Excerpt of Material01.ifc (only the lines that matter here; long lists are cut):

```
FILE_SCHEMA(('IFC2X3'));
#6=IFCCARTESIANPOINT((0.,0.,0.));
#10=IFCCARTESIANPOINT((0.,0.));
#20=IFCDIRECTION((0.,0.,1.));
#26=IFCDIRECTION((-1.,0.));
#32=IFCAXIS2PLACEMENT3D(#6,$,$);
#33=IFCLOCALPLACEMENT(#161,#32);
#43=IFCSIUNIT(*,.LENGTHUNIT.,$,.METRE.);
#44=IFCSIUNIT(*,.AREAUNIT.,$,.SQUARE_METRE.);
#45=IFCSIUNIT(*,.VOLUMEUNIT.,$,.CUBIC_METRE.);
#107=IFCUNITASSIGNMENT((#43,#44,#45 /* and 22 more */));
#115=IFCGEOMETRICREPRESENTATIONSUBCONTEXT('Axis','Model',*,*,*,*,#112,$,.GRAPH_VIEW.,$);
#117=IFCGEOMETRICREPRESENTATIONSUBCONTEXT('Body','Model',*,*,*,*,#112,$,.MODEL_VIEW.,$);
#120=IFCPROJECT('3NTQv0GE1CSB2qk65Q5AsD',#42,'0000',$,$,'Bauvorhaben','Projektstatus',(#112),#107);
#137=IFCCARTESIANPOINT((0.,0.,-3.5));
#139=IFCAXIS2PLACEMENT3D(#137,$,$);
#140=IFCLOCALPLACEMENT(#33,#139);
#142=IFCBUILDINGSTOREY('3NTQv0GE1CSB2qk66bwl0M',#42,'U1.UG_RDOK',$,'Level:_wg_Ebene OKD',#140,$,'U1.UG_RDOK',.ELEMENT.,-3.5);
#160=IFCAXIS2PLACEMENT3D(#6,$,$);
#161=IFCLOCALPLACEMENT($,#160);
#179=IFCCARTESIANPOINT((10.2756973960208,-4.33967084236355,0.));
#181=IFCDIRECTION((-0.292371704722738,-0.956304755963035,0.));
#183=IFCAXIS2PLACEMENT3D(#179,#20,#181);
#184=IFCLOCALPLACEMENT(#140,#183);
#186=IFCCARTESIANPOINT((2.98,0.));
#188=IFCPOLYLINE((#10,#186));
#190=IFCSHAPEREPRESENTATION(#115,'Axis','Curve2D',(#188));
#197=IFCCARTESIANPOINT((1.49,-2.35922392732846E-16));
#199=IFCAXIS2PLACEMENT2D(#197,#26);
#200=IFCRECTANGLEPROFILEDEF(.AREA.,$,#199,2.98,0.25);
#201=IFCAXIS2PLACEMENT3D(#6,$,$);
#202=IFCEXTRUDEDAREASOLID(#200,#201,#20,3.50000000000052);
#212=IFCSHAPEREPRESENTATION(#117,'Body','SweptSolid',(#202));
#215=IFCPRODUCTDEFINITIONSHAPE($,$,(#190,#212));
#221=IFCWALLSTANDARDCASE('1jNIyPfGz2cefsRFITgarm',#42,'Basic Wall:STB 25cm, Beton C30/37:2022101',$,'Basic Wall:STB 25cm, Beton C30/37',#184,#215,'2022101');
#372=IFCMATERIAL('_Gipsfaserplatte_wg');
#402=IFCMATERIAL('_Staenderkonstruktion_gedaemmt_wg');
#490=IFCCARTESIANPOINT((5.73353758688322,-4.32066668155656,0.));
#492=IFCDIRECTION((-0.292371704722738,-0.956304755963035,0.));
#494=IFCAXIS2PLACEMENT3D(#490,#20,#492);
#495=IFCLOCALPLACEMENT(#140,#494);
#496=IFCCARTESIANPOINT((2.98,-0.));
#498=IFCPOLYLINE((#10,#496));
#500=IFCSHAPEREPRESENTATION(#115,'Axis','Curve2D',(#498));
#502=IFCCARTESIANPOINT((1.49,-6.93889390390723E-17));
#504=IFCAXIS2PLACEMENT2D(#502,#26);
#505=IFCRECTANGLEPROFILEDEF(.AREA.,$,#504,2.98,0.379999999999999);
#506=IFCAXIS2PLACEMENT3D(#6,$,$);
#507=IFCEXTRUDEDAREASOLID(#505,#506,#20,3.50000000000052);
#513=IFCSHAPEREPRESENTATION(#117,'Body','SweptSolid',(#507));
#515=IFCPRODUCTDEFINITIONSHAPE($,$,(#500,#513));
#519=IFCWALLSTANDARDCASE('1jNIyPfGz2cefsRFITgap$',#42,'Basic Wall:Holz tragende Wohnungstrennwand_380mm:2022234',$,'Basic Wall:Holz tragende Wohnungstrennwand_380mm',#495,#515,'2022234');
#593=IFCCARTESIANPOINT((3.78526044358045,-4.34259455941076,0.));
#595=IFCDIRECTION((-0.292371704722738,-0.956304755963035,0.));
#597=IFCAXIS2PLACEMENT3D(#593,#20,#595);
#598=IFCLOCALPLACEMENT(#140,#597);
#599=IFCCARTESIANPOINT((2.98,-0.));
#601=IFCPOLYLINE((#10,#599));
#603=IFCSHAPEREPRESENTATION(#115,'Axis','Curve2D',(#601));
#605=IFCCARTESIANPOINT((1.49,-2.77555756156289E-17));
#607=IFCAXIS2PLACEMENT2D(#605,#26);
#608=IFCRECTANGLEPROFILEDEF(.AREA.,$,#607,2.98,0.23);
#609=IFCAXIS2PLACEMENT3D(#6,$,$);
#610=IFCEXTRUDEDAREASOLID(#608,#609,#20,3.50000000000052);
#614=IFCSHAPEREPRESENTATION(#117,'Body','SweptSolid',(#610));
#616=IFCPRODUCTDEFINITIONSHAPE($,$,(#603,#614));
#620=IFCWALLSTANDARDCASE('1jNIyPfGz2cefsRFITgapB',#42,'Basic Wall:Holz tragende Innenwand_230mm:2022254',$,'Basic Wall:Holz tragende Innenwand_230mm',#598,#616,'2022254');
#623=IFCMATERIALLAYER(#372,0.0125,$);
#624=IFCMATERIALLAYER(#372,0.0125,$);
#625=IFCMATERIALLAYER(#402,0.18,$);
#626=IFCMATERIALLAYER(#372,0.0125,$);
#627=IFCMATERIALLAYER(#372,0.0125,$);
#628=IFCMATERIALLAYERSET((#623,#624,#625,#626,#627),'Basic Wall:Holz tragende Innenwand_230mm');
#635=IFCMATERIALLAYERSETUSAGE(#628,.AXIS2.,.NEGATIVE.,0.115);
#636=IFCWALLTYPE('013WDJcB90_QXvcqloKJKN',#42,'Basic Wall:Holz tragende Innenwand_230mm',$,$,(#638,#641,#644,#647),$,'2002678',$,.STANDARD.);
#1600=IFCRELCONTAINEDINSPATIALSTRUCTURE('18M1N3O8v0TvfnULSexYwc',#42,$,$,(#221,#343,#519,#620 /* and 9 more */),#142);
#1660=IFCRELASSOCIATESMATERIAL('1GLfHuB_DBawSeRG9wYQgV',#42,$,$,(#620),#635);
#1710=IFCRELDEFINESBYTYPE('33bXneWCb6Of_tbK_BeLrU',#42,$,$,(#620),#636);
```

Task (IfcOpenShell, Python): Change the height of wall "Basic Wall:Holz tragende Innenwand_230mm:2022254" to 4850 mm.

```python
import ifcopenshell
import ifcopenshell.geom
import ifcopenshell.util.representation
import ifcopenshell.util.shape

model = ifcopenshell.open("Material01.ifc")
settings = ifcopenshell.geom.settings()


def volume(element):
    """Net volume in cubic metres, openings subtracted."""
    shape = ifcopenshell.geom.create_shape(settings, element)
    return ifcopenshell.util.shape.get_volume(shape.geometry)


wall = model.by_id(620)
before = volume(wall)

body = ifcopenshell.util.representation.get_representation(wall, "Model", "Body")
solid = body.Items[0]
old_height = solid.Depth
solid.Depth = 4.85
after = volume(wall)

print(f"height {old_height:g} -> {solid.Depth:g}, volume {before:.3f} -> {after:.3f} m3")

model.write("Material01_updated.ifc")
```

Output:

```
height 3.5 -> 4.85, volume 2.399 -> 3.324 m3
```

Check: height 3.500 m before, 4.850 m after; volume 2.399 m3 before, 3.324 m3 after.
